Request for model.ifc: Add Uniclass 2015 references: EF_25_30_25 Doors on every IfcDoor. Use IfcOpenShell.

First a look at what the model holds.

```python
import ifcopenshell

model = ifcopenshell.open("model.ifc")
print(model.schema)
print("classifications:", [c.Name for c in model.by_type("IfcClassification")])
for ifc_class in ("IfcDoor", "IfcRoof", "IfcStair", "IfcWall", "IfcWindow"):
    print(ifc_class, len(model.by_type(ifc_class)))
```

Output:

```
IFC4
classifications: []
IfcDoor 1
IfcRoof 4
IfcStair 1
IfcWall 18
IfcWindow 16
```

```python
import ifcopenshell
import ifcopenshell.api.classification

model = ifcopenshell.open("model.ifc")

system = ifcopenshell.api.classification.add_classification(model, classification="Uniclass 2015")

codes = {
    "IfcDoor": ("EF_25_30_25", "Doors"),
}
for ifc_class, (code, name) in codes.items():
    products = model.by_type(ifc_class)
    ifcopenshell.api.classification.add_reference(
        model, products=products, classification=system, identification=code, name=name
    )
    print(code, len(products))

model.write("model_rev.ifc")
```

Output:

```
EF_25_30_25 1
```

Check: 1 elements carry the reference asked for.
